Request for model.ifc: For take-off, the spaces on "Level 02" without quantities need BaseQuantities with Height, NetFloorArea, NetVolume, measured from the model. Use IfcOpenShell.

First a look at what the model holds.

```python
import ifcopenshell
import ifcopenshell.util.element
import ifcopenshell.util.unit

model = ifcopenshell.open("model.ifc")
print(model.schema)
for unit_type in ("LENGTHUNIT", "AREAUNIT", "VOLUMEUNIT"):
    print(unit_type, ifcopenshell.util.unit.calculate_unit_scale(model, unit_type))
storey = next(s for s in model.by_type("IfcBuildingStorey") if s.Name == "Level 02")
spaces = [e for e in ifcopenshell.util.element.get_decomposition(storey) if e.is_a("IfcSpace")]
for e in sorted(spaces, key=lambda e: e.id()):
    print(e.id(), e.is_a(), e.Name, list(ifcopenshell.util.element.get_psets(e, qtos_only=True)), sep=" | ")
```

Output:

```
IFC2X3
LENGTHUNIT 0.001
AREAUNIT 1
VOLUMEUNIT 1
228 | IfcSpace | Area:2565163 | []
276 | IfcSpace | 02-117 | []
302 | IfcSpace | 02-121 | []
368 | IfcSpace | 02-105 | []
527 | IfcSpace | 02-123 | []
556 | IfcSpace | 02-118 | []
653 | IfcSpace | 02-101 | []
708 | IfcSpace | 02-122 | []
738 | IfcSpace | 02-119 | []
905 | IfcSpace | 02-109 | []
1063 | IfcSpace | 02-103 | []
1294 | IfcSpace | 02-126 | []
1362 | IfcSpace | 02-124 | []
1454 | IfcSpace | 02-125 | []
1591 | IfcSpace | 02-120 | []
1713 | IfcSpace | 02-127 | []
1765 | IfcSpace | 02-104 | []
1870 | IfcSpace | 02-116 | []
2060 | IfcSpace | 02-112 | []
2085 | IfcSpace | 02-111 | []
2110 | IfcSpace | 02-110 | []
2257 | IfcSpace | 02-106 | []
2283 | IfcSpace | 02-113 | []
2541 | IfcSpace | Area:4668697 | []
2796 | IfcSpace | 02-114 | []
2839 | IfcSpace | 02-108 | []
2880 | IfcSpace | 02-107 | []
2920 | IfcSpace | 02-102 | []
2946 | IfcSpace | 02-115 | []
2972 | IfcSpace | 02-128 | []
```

```python
import ifcopenshell
import ifcopenshell.api.pset
import ifcopenshell.geom
import ifcopenshell.util.element
import ifcopenshell.util.shape
import ifcopenshell.util.unit

model = ifcopenshell.open("model.ifc")
unit_scale = ifcopenshell.util.unit.calculate_unit_scale(model)
area_scale = ifcopenshell.util.unit.calculate_unit_scale(model, "AREAUNIT")
volume_scale = ifcopenshell.util.unit.calculate_unit_scale(model, "VOLUMEUNIT")
settings = ifcopenshell.geom.settings()

storey = next(s for s in model.by_type("IfcBuildingStorey") if s.Name == "Level 02")
spaces = [e for e in ifcopenshell.util.element.get_decomposition(storey) if e.is_a("IfcSpace")]

for e in sorted(spaces, key=lambda e: e.id()):
    if ifcopenshell.util.element.get_psets(e, qtos_only=True, should_inherit=False):
        continue
    # Geometry comes back in metres, in the element's own axes.
    shape = ifcopenshell.geom.create_shape(settings, e)
    values = {
        "Height": ifcopenshell.util.shape.get_z(shape.geometry) / unit_scale,
        "NetFloorArea": ifcopenshell.util.shape.get_footprint_area(shape.geometry) / area_scale,
        "NetVolume": ifcopenshell.util.shape.get_volume(shape.geometry) / volume_scale,
    }
    qto = ifcopenshell.api.pset.add_qto(model, product=e, name="BaseQuantities")
    ifcopenshell.api.pset.edit_qto(model, qto=qto, properties=values)
    print(e.id(), {k: round(v, 3) for k, v in values.items()})

model.write("model-out.ifc")
```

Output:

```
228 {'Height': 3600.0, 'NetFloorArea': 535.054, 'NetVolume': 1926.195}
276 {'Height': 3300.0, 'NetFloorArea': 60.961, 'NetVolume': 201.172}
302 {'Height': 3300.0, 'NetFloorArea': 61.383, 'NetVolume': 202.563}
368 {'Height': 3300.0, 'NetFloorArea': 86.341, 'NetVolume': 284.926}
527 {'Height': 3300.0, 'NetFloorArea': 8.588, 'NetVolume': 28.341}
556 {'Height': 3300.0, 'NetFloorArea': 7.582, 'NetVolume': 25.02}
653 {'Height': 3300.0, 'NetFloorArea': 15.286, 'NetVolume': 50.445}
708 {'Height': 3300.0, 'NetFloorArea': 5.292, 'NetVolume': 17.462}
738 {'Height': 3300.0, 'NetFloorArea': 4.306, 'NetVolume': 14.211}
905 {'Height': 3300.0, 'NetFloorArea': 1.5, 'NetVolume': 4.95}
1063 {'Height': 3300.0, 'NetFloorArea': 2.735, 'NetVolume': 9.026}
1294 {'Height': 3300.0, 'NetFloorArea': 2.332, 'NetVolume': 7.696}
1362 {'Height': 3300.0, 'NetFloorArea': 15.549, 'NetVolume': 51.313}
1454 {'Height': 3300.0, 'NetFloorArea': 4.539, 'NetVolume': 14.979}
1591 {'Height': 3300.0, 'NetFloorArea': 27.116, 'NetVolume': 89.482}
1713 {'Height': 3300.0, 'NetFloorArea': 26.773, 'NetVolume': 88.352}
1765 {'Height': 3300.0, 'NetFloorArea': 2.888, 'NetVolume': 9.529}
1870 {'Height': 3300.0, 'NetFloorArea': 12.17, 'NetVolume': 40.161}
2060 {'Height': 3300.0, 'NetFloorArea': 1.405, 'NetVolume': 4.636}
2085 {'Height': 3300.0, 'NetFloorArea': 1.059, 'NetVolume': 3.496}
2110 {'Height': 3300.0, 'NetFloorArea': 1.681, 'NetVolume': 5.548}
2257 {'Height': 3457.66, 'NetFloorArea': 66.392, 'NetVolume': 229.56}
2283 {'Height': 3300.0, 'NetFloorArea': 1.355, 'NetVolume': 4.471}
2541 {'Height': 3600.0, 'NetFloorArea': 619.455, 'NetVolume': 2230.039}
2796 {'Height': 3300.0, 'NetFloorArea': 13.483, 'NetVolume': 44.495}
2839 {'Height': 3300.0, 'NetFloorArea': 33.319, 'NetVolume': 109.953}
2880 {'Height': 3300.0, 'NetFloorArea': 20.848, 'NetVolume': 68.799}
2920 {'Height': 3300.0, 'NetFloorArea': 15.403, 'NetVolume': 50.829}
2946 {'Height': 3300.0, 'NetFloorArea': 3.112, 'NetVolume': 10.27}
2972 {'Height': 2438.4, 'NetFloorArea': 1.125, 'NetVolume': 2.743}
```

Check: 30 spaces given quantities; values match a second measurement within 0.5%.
